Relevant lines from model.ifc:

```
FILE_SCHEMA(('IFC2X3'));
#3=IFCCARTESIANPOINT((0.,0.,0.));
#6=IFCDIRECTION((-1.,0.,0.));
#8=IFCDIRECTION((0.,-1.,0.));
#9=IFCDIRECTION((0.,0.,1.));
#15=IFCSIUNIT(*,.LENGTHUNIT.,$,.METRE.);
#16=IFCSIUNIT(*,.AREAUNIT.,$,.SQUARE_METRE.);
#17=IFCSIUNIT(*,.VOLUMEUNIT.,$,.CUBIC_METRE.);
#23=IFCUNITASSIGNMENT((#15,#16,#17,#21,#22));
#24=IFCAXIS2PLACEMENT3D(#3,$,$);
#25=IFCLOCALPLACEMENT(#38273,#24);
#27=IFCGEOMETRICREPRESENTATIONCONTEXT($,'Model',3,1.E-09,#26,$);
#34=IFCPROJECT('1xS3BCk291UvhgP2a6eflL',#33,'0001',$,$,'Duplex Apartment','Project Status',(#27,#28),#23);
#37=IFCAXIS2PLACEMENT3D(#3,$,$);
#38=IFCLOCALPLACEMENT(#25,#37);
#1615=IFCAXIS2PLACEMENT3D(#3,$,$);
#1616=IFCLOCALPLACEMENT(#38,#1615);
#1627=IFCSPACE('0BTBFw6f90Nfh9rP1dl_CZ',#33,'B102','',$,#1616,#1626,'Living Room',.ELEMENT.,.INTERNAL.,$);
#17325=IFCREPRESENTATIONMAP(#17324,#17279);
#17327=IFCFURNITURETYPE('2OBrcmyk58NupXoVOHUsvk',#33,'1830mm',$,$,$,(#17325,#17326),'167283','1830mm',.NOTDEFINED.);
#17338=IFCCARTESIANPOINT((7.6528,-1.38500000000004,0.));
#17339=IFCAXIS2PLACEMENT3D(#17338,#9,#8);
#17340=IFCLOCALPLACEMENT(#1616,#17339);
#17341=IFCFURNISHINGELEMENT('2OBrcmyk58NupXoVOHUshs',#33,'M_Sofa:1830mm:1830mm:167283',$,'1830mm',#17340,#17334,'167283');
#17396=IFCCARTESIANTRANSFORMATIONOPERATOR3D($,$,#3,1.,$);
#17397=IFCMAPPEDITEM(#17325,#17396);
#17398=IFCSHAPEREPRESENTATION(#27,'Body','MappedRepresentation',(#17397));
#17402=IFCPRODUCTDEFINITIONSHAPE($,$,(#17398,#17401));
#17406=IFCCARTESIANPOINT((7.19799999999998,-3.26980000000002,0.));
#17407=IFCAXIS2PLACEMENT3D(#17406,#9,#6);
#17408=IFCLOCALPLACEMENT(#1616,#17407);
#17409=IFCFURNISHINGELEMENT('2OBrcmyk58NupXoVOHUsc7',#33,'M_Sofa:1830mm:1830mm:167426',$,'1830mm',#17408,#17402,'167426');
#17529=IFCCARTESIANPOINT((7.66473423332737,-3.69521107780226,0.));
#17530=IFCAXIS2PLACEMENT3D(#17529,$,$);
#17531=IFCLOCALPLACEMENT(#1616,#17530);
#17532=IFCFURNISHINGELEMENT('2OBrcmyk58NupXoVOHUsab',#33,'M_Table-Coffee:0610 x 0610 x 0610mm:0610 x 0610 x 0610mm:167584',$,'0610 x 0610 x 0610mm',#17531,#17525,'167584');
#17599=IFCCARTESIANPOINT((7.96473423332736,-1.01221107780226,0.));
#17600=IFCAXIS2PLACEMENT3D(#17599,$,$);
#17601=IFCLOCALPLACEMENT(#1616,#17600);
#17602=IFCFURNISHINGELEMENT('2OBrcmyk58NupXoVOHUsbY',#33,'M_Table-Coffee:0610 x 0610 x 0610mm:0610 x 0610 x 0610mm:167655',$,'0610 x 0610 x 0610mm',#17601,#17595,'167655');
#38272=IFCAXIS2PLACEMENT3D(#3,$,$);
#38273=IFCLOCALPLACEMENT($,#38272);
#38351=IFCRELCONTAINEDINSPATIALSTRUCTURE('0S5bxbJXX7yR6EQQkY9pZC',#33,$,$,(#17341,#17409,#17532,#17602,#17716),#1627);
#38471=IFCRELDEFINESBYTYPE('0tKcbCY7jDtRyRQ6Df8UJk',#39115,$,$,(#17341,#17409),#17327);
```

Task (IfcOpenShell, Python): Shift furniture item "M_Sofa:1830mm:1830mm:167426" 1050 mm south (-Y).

```python
import ifcopenshell
import ifcopenshell.api.geometry
import ifcopenshell.util.placement
import ifcopenshell.util.unit

model = ifcopenshell.open("model.ifc")
unit_scale = ifcopenshell.util.unit.calculate_unit_scale(model)

item = model.by_guid("2OBrcmyk58NupXoVOHUsc7")
matrix = ifcopenshell.util.placement.get_local_placement(item.ObjectPlacement)
matrix[1, 3] -= 1.05 / unit_scale
ifcopenshell.api.geometry.edit_object_placement(model, product=item, matrix=matrix, is_si=False)

print(ifcopenshell.util.placement.get_local_placement(item.ObjectPlacement).round(3) + 0.0)

model.write("model_updated.ifc")
```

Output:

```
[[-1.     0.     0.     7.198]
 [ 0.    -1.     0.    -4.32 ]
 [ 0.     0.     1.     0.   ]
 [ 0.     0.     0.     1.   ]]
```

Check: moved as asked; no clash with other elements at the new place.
